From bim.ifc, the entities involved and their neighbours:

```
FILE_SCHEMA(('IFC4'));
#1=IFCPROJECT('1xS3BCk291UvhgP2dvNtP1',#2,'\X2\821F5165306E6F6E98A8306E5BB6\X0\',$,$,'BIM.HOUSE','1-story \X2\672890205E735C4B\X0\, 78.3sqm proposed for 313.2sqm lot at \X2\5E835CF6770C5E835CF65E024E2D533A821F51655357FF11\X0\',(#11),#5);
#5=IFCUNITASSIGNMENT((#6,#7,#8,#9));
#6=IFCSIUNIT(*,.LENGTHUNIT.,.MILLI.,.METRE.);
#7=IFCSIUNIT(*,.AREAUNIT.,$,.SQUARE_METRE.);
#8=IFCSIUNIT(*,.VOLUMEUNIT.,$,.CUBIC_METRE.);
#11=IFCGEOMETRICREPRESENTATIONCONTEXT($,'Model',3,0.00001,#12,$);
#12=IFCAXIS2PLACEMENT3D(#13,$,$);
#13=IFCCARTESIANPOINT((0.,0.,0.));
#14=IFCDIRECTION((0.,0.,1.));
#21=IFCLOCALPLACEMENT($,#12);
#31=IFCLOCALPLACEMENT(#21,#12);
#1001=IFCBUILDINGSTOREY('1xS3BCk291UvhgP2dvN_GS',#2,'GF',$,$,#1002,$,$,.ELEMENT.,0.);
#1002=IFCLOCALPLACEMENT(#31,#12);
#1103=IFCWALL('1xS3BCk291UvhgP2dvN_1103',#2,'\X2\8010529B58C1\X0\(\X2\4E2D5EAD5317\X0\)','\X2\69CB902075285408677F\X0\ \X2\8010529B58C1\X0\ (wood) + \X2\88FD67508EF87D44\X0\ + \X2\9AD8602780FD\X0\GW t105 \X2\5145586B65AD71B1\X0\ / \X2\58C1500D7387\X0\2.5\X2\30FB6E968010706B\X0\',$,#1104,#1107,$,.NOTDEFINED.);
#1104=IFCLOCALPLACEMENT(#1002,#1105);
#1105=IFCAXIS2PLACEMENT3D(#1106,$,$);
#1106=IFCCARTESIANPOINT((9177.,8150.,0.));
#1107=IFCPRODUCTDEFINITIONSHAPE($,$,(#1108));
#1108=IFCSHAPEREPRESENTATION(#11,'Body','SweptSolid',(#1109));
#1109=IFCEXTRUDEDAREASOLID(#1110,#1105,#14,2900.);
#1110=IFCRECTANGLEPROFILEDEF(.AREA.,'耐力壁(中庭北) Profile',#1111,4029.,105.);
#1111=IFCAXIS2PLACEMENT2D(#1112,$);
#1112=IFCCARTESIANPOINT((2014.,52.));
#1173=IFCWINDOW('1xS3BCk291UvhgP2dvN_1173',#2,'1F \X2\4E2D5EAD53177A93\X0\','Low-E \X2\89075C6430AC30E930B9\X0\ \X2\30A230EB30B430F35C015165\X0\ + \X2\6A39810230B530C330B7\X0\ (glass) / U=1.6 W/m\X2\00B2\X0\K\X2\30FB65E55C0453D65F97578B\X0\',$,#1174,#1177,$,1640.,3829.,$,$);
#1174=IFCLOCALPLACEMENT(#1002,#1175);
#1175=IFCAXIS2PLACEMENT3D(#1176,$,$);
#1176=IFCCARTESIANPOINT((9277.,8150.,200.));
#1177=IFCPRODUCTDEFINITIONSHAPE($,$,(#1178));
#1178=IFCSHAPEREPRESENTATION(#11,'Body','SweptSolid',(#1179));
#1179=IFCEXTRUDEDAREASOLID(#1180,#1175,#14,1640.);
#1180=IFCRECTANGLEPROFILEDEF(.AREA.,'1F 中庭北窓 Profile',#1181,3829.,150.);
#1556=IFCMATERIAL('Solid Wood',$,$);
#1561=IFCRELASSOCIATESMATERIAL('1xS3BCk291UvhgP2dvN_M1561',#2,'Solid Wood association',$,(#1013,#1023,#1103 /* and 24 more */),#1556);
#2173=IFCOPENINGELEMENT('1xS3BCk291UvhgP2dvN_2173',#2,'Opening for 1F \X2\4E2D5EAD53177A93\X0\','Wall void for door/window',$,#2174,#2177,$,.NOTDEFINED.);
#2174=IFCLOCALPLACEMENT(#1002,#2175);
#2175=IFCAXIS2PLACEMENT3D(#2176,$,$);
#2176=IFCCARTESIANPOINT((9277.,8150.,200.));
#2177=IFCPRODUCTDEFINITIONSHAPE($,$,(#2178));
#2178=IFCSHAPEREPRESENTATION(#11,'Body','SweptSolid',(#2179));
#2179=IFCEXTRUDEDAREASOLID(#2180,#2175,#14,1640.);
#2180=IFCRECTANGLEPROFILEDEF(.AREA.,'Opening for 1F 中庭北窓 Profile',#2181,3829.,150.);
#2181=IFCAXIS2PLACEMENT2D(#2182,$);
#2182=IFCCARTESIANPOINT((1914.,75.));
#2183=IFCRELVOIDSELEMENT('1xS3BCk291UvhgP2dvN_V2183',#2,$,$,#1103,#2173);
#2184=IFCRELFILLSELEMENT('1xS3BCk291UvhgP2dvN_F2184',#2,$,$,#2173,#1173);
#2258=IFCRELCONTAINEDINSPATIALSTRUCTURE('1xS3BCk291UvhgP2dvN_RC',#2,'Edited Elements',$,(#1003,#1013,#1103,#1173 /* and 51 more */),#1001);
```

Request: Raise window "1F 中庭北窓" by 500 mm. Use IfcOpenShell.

```python
import numpy as np
import ifcopenshell
import ifcopenshell.api.geometry
import ifcopenshell.util.placement
import ifcopenshell.util.unit

model = ifcopenshell.open("bim.ifc")
unit_scale = ifcopenshell.util.unit.calculate_unit_scale(model)

window = model.by_guid("1xS3BCk291UvhgP2dvN_1173")
opening = window.FillsVoids[0].RelatingOpeningElement
dz = 0.5 / unit_scale

shift = np.array([0.0, 0.0, dz])
# The window is not placed relative to its opening, so move both.
for product in (opening, window):
    matrix = ifcopenshell.util.placement.get_local_placement(product.ObjectPlacement)
    matrix[:3, 3] += shift
    ifcopenshell.api.geometry.edit_object_placement(model, product=product, matrix=matrix, is_si=False)

print(f"moved by {dz * unit_scale:+.3f} m")

model.write("bim_v2.ifc")
```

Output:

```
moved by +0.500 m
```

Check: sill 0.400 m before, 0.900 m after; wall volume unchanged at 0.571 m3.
